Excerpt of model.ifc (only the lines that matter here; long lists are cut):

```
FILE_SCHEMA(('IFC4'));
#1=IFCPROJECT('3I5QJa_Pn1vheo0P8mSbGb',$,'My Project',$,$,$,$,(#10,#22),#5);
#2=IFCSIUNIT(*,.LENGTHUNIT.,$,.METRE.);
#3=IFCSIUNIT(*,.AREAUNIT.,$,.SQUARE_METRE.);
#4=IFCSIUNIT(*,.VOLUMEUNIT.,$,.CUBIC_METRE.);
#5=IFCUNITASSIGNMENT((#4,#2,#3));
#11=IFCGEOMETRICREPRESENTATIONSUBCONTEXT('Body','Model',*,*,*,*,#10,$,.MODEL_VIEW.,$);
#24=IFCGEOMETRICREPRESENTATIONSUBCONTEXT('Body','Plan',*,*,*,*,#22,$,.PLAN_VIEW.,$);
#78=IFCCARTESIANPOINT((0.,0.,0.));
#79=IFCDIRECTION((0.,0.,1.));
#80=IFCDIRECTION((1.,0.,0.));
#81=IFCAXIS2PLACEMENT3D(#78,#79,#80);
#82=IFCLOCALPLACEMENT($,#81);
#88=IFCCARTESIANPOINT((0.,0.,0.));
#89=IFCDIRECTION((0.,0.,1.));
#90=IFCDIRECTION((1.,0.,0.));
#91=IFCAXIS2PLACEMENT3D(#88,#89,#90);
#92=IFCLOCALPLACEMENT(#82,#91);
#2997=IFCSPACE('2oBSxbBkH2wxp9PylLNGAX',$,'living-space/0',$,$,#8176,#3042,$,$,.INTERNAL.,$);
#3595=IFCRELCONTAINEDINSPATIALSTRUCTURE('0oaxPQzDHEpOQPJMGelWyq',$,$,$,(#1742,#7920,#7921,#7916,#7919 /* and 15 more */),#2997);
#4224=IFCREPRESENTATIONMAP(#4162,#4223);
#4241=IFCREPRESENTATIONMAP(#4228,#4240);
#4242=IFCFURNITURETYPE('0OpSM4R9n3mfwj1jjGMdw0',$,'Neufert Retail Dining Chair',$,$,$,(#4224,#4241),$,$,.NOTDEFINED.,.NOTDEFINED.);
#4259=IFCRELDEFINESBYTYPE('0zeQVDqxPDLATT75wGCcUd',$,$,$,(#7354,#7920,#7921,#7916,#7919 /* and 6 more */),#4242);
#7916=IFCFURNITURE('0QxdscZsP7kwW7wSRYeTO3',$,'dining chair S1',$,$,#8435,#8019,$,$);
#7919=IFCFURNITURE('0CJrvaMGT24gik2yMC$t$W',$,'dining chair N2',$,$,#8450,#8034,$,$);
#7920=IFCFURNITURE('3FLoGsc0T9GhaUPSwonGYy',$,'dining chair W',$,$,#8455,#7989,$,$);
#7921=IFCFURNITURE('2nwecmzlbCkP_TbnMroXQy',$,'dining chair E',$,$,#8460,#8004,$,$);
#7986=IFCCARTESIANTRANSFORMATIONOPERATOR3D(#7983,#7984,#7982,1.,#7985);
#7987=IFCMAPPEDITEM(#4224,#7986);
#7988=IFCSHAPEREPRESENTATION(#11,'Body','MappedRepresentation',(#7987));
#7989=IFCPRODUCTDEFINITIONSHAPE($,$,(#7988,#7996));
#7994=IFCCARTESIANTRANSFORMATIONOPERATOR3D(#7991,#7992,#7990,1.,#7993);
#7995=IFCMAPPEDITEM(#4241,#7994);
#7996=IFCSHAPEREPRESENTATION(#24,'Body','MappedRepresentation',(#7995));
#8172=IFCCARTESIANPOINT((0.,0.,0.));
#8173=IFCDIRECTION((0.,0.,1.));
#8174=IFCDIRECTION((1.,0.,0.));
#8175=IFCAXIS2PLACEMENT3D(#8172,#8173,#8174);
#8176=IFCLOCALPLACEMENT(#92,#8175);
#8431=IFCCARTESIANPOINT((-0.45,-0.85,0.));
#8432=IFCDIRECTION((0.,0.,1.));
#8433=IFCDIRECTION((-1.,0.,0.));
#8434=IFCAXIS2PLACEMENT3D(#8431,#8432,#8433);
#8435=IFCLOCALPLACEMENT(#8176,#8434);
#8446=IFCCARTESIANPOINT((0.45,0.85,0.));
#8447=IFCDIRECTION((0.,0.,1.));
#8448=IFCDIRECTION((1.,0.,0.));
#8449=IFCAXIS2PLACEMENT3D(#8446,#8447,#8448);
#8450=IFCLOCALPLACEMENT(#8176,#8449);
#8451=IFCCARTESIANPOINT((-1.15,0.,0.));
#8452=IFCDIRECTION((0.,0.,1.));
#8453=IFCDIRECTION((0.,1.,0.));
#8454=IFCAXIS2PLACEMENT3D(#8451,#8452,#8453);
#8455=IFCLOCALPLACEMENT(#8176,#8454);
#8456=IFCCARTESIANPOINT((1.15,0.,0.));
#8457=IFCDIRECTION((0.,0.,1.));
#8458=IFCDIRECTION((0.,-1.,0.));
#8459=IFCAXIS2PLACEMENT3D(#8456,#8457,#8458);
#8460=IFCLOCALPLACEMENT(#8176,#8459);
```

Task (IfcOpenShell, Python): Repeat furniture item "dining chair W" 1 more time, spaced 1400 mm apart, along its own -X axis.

```python
import ifcopenshell
import ifcopenshell.api.geometry
import ifcopenshell.api.root
import ifcopenshell.util.element
import ifcopenshell.util.placement
import ifcopenshell.util.unit

model = ifcopenshell.open("model.ifc")
unit_scale = ifcopenshell.util.unit.calculate_unit_scale(model)

source = model.by_guid("3FLoGsc0T9GhaUPSwonGYy")
base = ifcopenshell.util.placement.get_local_placement(source.ObjectPlacement)
step = -base[:3, 0] * 1.4 / unit_scale

for i in range(1, 2):
    copy = ifcopenshell.api.root.copy_class(model, product=source)
    copy.Representation = ifcopenshell.util.element.copy_deep(
        model, source.Representation, exclude=["IfcGeometricRepresentationContext", "IfcRepresentationMap"]
    )
    matrix = base.copy()
    matrix[:3, 3] += i * step
    print("added at", matrix[:3, 3].round(3) + 0.0)
    ifcopenshell.api.geometry.edit_object_placement(model, product=copy, matrix=matrix, is_si=False)

model.write("model_updated.ifc")
```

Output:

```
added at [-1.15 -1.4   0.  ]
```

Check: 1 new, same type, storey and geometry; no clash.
